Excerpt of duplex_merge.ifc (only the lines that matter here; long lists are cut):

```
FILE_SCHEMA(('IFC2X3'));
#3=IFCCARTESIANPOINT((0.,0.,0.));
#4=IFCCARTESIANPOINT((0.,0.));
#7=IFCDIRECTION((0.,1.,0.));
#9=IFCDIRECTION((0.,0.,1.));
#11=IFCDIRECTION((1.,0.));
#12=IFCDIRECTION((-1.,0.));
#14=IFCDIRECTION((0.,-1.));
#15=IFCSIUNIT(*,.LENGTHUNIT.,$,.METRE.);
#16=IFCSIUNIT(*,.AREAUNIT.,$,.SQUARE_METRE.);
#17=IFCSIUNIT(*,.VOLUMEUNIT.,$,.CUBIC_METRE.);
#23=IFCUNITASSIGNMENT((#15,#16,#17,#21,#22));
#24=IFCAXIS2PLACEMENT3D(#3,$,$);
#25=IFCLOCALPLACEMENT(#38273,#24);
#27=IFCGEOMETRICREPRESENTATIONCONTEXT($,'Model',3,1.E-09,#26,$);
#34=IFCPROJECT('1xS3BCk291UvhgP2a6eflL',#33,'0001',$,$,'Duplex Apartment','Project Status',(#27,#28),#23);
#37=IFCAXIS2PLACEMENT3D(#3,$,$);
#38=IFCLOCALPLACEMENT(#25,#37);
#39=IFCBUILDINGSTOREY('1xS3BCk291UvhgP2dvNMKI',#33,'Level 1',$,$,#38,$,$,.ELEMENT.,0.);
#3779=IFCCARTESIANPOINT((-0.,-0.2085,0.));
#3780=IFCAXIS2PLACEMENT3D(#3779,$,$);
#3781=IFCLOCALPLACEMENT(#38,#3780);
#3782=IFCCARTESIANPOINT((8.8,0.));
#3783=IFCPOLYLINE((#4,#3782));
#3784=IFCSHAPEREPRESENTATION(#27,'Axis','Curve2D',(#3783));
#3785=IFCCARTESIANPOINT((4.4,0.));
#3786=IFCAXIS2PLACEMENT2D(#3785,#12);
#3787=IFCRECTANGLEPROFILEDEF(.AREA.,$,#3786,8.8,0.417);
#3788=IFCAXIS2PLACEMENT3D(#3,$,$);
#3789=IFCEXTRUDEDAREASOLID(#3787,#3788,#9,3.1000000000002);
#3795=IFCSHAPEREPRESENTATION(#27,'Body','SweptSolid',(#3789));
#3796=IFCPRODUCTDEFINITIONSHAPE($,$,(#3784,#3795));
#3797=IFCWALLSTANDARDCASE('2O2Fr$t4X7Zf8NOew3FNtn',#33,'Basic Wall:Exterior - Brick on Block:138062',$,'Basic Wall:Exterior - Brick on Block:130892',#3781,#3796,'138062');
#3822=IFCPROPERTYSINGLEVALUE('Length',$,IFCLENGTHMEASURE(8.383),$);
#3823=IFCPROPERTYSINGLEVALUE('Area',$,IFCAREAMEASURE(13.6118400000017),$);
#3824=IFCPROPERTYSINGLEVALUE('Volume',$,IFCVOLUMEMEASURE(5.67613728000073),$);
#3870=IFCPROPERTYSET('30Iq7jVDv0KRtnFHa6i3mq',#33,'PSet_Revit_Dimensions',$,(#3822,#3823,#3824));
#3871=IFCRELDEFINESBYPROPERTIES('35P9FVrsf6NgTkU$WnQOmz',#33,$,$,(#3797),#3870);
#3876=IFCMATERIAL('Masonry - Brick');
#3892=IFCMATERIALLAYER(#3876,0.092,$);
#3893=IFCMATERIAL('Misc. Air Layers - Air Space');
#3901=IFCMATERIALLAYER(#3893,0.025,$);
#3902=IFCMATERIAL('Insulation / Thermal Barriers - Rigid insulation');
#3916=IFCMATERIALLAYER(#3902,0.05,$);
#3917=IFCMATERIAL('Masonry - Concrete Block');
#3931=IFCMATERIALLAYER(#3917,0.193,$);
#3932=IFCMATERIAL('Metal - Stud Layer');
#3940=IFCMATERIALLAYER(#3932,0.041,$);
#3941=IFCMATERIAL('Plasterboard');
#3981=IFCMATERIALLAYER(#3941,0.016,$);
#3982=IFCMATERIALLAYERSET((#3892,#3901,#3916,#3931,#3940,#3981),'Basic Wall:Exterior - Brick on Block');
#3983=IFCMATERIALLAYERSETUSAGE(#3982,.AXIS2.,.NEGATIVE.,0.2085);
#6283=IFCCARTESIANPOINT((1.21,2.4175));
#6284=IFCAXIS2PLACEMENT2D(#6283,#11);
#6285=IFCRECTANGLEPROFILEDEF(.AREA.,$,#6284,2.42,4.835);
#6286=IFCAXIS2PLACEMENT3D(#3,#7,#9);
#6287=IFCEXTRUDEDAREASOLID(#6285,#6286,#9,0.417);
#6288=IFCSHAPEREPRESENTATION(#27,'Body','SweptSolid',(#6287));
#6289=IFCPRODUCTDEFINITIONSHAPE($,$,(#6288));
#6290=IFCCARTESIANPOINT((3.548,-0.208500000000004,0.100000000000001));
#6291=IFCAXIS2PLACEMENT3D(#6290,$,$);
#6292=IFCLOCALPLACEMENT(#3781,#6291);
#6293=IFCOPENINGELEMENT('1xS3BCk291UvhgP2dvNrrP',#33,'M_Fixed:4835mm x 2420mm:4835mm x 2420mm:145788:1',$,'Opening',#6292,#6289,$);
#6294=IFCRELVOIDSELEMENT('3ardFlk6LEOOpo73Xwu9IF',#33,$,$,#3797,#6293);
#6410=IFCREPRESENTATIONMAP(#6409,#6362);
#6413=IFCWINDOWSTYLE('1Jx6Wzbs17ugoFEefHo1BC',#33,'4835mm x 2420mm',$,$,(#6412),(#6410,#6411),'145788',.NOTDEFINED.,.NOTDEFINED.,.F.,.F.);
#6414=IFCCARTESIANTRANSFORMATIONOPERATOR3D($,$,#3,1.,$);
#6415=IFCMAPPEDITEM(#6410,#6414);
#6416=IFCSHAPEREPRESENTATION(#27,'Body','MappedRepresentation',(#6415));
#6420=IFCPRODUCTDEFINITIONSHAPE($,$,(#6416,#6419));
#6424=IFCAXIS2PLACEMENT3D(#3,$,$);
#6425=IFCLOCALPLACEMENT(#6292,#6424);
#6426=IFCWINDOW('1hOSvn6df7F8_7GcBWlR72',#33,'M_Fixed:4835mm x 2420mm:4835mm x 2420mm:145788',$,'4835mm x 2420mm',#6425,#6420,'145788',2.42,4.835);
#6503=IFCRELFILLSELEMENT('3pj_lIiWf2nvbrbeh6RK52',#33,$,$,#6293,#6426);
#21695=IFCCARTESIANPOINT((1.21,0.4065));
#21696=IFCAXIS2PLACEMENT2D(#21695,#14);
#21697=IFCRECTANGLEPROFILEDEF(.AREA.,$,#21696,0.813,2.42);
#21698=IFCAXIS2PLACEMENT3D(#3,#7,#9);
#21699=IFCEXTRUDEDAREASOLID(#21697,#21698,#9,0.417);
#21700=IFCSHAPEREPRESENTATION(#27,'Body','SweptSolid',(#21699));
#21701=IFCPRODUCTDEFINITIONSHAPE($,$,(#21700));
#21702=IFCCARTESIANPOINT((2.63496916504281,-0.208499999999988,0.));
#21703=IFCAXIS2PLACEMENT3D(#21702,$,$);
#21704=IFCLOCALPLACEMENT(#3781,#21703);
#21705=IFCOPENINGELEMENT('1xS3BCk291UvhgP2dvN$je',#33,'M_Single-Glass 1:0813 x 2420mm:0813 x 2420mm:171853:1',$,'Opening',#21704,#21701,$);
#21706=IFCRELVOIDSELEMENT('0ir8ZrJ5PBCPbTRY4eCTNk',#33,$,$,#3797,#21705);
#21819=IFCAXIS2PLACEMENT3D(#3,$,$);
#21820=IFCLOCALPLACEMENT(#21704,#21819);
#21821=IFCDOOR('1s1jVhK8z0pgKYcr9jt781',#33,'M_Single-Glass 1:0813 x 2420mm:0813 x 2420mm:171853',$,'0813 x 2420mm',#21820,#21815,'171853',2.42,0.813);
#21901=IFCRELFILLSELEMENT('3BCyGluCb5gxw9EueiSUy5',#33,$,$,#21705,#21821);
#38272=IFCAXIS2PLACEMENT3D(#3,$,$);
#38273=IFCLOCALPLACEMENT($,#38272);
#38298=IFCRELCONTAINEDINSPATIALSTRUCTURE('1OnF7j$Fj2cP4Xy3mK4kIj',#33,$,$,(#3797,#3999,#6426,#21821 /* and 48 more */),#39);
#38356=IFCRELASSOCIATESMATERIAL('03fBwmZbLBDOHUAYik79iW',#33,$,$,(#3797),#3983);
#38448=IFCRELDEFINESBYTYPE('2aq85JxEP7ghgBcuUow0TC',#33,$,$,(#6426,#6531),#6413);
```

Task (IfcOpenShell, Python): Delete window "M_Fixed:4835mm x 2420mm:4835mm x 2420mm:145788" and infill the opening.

```python
import ifcopenshell
import ifcopenshell.api.feature
import ifcopenshell.api.pset
import ifcopenshell.api.root
import ifcopenshell.geom
import ifcopenshell.util.element
import ifcopenshell.util.shape
import ifcopenshell.util.unit

model = ifcopenshell.open("duplex_merge.ifc")
area_scale = ifcopenshell.util.unit.calculate_unit_scale(model, "AREAUNIT")
volume_scale = ifcopenshell.util.unit.calculate_unit_scale(model, "VOLUMEUNIT")
settings = ifcopenshell.geom.settings()


def volume(element):
    """Net volume in cubic metres, openings subtracted."""
    shape = ifcopenshell.geom.create_shape(settings, element)
    return ifcopenshell.util.shape.get_volume(shape.geometry)


window = model.by_id(6426)
opening = window.FillsVoids[0].RelatingOpeningElement
wall = opening.VoidsElements[0].RelatingBuildingElement
before = volume(wall)

ifcopenshell.api.root.remove_product(model, product=window)
ifcopenshell.api.feature.remove_feature(model, feature=opening)

after = volume(wall)
thickness = 0.417  # wall thickness in metres

# Update the wall's stored quantities.
pset = model.by_id(ifcopenshell.util.element.get_pset(wall, "PSet_Revit_Dimensions", should_inherit=False)["id"])
ifcopenshell.api.pset.edit_pset(model, pset=pset, properties={
    "Area": model.create_entity("IfcAreaMeasure", after / thickness / area_scale),
    "Volume": model.create_entity("IfcVolumeMeasure", after / volume_scale),
})

print(f"wall volume {before:.3f} -> {after:.3f} m3")

model.write("duplex_merge_v2.ifc")
```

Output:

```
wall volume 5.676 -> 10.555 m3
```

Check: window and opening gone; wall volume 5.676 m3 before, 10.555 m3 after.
